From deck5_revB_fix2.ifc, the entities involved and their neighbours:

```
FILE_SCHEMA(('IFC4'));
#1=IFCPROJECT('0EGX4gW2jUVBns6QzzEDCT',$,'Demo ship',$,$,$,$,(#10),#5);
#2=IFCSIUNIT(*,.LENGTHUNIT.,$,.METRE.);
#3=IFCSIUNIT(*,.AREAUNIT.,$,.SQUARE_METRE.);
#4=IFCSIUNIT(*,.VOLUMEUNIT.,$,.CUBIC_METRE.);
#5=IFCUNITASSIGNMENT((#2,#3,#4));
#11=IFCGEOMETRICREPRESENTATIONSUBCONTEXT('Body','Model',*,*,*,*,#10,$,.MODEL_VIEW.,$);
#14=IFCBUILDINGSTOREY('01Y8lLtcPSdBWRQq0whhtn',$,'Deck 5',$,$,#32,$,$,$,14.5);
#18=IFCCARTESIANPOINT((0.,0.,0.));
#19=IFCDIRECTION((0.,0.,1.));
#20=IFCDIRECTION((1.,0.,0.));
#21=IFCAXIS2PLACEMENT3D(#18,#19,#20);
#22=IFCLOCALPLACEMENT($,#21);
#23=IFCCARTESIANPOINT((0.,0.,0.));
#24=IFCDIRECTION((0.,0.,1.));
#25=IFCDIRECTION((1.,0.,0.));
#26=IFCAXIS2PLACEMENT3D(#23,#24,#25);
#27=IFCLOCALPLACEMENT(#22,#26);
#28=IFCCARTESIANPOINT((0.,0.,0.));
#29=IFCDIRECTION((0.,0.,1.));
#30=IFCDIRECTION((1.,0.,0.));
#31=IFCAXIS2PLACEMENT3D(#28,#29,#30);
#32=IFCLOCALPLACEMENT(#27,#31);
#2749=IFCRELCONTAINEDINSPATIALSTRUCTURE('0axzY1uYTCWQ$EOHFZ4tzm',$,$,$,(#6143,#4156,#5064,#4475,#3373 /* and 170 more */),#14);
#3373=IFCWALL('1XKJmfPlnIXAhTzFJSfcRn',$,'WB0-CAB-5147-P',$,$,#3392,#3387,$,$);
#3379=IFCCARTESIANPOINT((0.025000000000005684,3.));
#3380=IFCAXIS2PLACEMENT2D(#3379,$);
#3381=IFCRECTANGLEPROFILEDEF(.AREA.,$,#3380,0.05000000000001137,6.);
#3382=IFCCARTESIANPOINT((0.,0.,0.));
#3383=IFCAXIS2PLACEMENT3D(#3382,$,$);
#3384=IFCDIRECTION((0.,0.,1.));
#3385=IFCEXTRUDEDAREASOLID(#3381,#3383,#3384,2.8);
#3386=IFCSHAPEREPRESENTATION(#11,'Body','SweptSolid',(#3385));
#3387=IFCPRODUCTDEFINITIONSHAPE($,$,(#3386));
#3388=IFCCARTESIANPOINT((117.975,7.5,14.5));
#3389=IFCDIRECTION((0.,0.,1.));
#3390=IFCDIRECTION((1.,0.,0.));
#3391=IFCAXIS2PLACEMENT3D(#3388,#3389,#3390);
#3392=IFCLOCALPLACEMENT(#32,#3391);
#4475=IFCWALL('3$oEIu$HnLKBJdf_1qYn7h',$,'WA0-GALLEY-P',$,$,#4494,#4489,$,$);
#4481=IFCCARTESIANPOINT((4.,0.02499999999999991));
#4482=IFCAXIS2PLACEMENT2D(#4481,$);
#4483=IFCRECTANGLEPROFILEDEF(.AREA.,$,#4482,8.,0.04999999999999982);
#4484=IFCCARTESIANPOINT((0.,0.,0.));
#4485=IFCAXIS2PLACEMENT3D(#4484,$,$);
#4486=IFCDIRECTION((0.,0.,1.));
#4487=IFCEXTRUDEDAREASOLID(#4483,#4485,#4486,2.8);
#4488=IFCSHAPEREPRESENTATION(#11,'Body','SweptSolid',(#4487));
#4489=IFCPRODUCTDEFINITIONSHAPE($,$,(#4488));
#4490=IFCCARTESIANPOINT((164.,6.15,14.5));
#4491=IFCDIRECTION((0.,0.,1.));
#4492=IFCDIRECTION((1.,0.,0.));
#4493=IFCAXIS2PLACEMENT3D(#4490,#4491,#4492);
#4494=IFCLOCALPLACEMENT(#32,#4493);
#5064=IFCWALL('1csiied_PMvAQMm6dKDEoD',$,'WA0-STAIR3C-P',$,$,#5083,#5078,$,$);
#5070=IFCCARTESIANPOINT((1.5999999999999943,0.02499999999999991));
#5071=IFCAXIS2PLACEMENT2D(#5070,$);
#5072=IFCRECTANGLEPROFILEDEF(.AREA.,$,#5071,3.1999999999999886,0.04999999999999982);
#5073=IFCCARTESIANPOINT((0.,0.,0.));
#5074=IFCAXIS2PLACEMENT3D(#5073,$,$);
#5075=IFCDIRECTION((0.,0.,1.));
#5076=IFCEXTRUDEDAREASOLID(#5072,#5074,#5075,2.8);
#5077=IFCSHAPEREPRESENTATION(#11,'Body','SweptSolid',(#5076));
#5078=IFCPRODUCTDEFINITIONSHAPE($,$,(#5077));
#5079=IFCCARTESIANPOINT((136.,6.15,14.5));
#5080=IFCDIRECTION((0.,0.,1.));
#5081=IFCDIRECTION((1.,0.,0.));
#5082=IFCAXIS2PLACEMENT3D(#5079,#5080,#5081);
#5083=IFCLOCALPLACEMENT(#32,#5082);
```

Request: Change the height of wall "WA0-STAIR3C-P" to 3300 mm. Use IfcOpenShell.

```python
import ifcopenshell
import ifcopenshell.geom
import ifcopenshell.util.representation
import ifcopenshell.util.shape

model = ifcopenshell.open("deck5_revB_fix2.ifc")
settings = ifcopenshell.geom.settings()


def volume(element):
    """Net volume in cubic metres, openings subtracted."""
    shape = ifcopenshell.geom.create_shape(settings, element)
    return ifcopenshell.util.shape.get_volume(shape.geometry)


wall = model.by_guid("1csiied_PMvAQMm6dKDEoD")
before = volume(wall)

body = ifcopenshell.util.representation.get_representation(wall, "Model", "Body")
solid = body.Items[0]
old_height = solid.Depth
solid.Depth = 3.3
after = volume(wall)

print(f"height {old_height:g} -> {solid.Depth:g}, volume {before:.3f} -> {after:.3f} m3")

model.write("deck5_revB_fix2-out.ifc")
```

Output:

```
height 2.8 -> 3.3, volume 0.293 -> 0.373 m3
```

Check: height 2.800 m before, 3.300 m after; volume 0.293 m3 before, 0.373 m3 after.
